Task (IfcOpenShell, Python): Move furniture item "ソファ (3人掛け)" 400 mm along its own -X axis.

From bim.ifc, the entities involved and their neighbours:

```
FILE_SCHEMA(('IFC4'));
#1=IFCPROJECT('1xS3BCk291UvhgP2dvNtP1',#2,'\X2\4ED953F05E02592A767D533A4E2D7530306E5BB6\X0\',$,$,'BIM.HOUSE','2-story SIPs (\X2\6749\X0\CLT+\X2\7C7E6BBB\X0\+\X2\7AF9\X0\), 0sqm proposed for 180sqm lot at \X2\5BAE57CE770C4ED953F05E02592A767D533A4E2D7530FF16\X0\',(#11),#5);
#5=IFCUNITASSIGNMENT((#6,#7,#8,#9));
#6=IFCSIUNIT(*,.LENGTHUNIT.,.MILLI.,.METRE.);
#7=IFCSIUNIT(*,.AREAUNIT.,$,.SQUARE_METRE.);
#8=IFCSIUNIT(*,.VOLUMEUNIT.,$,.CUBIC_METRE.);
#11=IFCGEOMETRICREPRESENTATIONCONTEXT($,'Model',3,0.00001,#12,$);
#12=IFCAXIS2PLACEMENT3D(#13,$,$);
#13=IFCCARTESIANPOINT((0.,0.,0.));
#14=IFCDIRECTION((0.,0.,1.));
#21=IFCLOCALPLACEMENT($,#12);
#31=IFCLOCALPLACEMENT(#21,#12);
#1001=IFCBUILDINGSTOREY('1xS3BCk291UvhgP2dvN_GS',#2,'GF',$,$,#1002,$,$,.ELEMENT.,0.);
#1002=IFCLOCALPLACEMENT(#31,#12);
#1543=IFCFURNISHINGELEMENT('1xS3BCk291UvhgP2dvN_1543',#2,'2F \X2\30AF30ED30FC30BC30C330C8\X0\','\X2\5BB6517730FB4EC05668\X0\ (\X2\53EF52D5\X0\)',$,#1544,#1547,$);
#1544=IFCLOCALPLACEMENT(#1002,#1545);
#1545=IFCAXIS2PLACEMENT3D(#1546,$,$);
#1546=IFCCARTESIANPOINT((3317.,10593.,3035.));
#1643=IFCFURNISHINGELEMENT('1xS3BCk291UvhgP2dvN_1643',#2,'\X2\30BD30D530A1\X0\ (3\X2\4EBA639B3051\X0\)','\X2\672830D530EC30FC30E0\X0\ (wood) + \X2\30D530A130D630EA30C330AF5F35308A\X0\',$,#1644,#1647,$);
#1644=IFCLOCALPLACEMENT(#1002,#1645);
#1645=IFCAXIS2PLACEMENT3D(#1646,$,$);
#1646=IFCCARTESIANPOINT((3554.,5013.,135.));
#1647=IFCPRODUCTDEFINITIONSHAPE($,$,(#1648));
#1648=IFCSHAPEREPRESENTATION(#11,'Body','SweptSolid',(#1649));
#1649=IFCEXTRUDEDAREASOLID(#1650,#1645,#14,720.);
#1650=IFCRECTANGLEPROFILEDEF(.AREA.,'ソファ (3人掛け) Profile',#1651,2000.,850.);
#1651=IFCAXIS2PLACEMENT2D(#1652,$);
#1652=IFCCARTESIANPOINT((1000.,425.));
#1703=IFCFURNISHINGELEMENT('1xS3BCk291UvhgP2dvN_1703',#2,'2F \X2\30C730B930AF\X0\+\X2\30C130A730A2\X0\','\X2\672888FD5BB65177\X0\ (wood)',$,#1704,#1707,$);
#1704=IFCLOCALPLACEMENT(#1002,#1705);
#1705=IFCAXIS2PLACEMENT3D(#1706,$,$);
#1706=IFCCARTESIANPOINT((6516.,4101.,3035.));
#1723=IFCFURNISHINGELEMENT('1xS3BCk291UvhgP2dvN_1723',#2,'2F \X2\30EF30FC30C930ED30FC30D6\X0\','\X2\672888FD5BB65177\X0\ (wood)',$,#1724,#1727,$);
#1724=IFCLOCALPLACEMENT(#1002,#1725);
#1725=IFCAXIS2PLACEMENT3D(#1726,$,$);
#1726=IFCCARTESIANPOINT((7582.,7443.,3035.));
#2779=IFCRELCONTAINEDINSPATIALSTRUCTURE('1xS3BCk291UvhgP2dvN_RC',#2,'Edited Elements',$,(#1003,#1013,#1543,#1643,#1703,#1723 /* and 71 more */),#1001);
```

```python
import ifcopenshell
import ifcopenshell.api.geometry
import ifcopenshell.util.placement

model = ifcopenshell.open("bim.ifc")

item = model.by_guid("1xS3BCk291UvhgP2dvN_1643")
matrix = ifcopenshell.util.placement.get_local_placement(item.ObjectPlacement)
matrix[:3, 3] -= matrix[:3, 0] * 400.0
ifcopenshell.api.geometry.edit_object_placement(model, product=item, matrix=matrix, is_si=False)

print(ifcopenshell.util.placement.get_local_placement(item.ObjectPlacement).round(3) + 0.0)

model.write("bim_v2.ifc")
```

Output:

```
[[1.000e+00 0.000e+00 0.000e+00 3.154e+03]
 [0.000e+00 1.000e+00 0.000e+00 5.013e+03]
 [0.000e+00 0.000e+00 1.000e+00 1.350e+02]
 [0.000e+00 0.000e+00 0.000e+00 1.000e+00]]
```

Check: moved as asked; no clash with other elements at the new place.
